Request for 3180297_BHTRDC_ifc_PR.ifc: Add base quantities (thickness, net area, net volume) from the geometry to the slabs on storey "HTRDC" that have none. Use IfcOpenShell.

First a look at what the model holds.

```python
import ifcopenshell
import ifcopenshell.util.element
import ifcopenshell.util.unit

model = ifcopenshell.open("3180297_BHTRDC_ifc_PR.ifc")
print(model.schema)
for unit_type in ("LENGTHUNIT", "AREAUNIT", "VOLUMEUNIT"):
    print(unit_type, ifcopenshell.util.unit.calculate_unit_scale(model, unit_type))
storey = next(s for s in model.by_type("IfcBuildingStorey") if s.Name == "HTRDC")
slabs = [e for e in ifcopenshell.util.element.get_decomposition(storey) if e.is_a("IfcSlab")]
for e in sorted(slabs, key=lambda e: e.id()):
    print(e.id(), e.is_a(), e.Name, list(ifcopenshell.util.element.get_psets(e, qtos_only=True)), sep=" | ")
```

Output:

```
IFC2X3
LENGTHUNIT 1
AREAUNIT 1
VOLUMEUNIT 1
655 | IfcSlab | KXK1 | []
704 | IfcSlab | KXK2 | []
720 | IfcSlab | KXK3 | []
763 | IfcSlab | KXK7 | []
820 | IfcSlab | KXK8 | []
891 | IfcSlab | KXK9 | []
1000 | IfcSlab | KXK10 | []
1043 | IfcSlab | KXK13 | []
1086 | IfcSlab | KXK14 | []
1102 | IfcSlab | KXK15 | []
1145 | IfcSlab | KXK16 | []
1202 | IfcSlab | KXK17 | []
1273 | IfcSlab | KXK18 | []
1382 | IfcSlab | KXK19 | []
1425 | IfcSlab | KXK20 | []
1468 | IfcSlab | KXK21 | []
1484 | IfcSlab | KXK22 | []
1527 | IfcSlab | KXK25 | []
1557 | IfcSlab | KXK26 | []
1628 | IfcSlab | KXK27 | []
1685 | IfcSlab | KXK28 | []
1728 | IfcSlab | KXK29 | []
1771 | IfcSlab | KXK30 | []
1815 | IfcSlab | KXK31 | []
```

```python
import ifcopenshell
import ifcopenshell.api.pset
import ifcopenshell.geom
import ifcopenshell.util.element
import ifcopenshell.util.shape
import ifcopenshell.util.unit

model = ifcopenshell.open("3180297_BHTRDC_ifc_PR.ifc")
unit_scale = ifcopenshell.util.unit.calculate_unit_scale(model)
area_scale = ifcopenshell.util.unit.calculate_unit_scale(model, "AREAUNIT")
volume_scale = ifcopenshell.util.unit.calculate_unit_scale(model, "VOLUMEUNIT")
settings = ifcopenshell.geom.settings()

storey = next(s for s in model.by_type("IfcBuildingStorey") if s.Name == "HTRDC")
slabs = [e for e in ifcopenshell.util.element.get_decomposition(storey) if e.is_a("IfcSlab")]

for e in sorted(slabs, key=lambda e: e.id()):
    if ifcopenshell.util.element.get_psets(e, qtos_only=True, should_inherit=False):
        continue
    # Geometry comes back in metres, in the element's own axes.
    shape = ifcopenshell.geom.create_shape(settings, e)
    values = {
        "Width": ifcopenshell.util.shape.get_z(shape.geometry) / unit_scale,
        "NetArea": ifcopenshell.util.shape.get_footprint_area(shape.geometry) / area_scale,
        "NetVolume": ifcopenshell.util.shape.get_volume(shape.geometry) / volume_scale,
    }
    qto = ifcopenshell.api.pset.add_qto(model, product=e, name="BaseQuantities")
    ifcopenshell.api.pset.edit_qto(model, qto=qto, properties=values)
    print(e.id(), {k: round(v, 3) for k, v in values.items()})

model.write("3180297_BHTRDC_ifc_PR_edited.ifc")
```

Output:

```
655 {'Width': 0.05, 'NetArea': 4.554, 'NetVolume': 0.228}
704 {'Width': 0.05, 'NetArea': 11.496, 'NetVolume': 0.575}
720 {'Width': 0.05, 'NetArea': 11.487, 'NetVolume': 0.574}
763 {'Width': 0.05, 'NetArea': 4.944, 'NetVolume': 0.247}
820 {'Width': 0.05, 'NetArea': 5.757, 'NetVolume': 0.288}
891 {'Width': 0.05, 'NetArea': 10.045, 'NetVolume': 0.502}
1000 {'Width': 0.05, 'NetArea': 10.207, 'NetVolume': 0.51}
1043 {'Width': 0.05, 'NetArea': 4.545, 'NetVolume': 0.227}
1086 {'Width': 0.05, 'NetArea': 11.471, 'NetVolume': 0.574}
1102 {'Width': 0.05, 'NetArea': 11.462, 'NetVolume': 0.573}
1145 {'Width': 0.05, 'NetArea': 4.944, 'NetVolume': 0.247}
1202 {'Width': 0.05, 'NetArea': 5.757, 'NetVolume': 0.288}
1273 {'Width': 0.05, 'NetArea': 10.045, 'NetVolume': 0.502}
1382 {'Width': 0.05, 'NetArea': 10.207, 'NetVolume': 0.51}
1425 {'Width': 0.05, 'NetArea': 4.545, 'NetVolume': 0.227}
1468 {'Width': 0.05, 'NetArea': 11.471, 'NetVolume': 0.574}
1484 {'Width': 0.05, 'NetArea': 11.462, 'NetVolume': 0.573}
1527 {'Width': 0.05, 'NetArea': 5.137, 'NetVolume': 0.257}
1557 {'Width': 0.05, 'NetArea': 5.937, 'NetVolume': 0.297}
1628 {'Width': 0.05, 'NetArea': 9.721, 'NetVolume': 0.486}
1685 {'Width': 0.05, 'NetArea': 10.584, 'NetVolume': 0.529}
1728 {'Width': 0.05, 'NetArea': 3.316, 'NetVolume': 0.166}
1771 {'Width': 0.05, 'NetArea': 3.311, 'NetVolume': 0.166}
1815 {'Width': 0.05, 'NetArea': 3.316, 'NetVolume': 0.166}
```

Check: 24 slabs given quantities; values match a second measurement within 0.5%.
